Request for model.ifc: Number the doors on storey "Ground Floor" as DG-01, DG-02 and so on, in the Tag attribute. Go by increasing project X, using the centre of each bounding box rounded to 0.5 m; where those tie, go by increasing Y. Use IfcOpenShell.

First a look at what the model holds.

```python
import ifcopenshell
import ifcopenshell.util.element
import ifcopenshell.util.placement

model = ifcopenshell.open("model.ifc")
print(model.schema)
storey = next(s for s in model.by_type("IfcBuildingStorey") if s.Name == "Ground Floor")
doors = [e for e in ifcopenshell.util.element.get_decomposition(storey) if e.is_a("IfcDoor")]
for e in sorted(doors, key=lambda e: e.id()):
    origin = ifcopenshell.util.placement.get_local_placement(e.ObjectPlacement)[:3, 3]
    print(e.id(), e.Tag, e.Name, origin.round(2) + 0.0, sep=" | ")
```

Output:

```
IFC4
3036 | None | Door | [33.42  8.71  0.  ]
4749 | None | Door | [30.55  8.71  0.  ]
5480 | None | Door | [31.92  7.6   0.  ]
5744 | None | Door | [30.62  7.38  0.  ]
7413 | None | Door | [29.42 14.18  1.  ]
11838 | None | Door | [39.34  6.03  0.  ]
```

```python
import ifcopenshell
import ifcopenshell.geom
import ifcopenshell.util.element
import ifcopenshell.util.shape

model = ifcopenshell.open("model.ifc")
settings = ifcopenshell.geom.settings()
settings.set("use-world-coords", True)


def centre(element):
    shape = ifcopenshell.geom.create_shape(settings, element)
    return ifcopenshell.util.shape.get_bbox_centroid(shape.geometry)


storey = next(s for s in model.by_type("IfcBuildingStorey") if s.Name == "Ground Floor")
doors = [e for e in ifcopenshell.util.element.get_decomposition(storey) if e.is_a("IfcDoor")]

# Insertion points can sit at a corner or the storey origin, so sort by the geometry (in metres).
centres = {e: centre(e) for e in doors}
doors.sort(key=lambda e: (round(centres[e][0] / 0.5), centres[e][1]))

for i, e in enumerate(doors, start=1):
    number = f"DG-{i:02d}"
    e.Tag = number
    print(e.id(), number)

model.write("model_updated.ifc")
```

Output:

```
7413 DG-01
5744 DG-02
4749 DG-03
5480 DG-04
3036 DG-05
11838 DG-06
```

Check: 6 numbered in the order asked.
